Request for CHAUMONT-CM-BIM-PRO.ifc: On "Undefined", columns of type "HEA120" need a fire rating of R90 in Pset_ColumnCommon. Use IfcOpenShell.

First a look at what the model holds.

```python
import ifcopenshell
import ifcopenshell.util.element

model = ifcopenshell.open("CHAUMONT-CM-BIM-PRO.ifc")
print(model.schema)
storey = next(s for s in model.by_type("IfcBuildingStorey") if s.Name == "Undefined")
columns = [e for e in ifcopenshell.util.element.get_decomposition(storey) if e.is_a("IfcColumn")]
seen = {}
for e in columns:
    element_type = ifcopenshell.util.element.get_type(e)
    key = (element_type.Name if element_type != e and element_type else None, ifcopenshell.util.element.get_pset(e, "Pset_ColumnCommon", "FireRating"))
    seen[key] = seen.get(key, 0) + 1
for (name, value), count in sorted(seen.items(), key=str):
    print(count, "x", name, "|", value)
```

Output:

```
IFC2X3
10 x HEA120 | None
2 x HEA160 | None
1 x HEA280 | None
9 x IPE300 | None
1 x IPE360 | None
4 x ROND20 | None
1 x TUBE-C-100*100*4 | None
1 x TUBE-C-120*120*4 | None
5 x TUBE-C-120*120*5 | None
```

```python
import ifcopenshell
import ifcopenshell.api.pset
import ifcopenshell.util.element

model = ifcopenshell.open("CHAUMONT-CM-BIM-PRO.ifc")

storey = next(s for s in model.by_type("IfcBuildingStorey") if s.Name == "Undefined")
columns = [e for e in ifcopenshell.util.element.get_decomposition(storey) if e.is_a("IfcColumn")]

count = 0
for e in columns:
    element_type = ifcopenshell.util.element.get_type(e)
    if element_type in (None, e) or element_type.Name != "HEA120":
        continue
    found = ifcopenshell.util.element.get_pset(e, "Pset_ColumnCommon", should_inherit=False)
    if found:
        pset = model.by_id(found["id"])
        if len(ifcopenshell.util.element.get_elements_by_pset(pset)) > 1:
            pset = ifcopenshell.api.pset.unshare_pset(model, products=[e], pset=pset)[0]
    else:
        pset = ifcopenshell.api.pset.add_pset(model, product=e, name="Pset_ColumnCommon")
    ifcopenshell.api.pset.edit_pset(model, pset=pset, properties={"FireRating": "R90"})
    count += 1

print(count, "columns updated")

model.write("CHAUMONT-CM-BIM-PRO-out.ifc")
```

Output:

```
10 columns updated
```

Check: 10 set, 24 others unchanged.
